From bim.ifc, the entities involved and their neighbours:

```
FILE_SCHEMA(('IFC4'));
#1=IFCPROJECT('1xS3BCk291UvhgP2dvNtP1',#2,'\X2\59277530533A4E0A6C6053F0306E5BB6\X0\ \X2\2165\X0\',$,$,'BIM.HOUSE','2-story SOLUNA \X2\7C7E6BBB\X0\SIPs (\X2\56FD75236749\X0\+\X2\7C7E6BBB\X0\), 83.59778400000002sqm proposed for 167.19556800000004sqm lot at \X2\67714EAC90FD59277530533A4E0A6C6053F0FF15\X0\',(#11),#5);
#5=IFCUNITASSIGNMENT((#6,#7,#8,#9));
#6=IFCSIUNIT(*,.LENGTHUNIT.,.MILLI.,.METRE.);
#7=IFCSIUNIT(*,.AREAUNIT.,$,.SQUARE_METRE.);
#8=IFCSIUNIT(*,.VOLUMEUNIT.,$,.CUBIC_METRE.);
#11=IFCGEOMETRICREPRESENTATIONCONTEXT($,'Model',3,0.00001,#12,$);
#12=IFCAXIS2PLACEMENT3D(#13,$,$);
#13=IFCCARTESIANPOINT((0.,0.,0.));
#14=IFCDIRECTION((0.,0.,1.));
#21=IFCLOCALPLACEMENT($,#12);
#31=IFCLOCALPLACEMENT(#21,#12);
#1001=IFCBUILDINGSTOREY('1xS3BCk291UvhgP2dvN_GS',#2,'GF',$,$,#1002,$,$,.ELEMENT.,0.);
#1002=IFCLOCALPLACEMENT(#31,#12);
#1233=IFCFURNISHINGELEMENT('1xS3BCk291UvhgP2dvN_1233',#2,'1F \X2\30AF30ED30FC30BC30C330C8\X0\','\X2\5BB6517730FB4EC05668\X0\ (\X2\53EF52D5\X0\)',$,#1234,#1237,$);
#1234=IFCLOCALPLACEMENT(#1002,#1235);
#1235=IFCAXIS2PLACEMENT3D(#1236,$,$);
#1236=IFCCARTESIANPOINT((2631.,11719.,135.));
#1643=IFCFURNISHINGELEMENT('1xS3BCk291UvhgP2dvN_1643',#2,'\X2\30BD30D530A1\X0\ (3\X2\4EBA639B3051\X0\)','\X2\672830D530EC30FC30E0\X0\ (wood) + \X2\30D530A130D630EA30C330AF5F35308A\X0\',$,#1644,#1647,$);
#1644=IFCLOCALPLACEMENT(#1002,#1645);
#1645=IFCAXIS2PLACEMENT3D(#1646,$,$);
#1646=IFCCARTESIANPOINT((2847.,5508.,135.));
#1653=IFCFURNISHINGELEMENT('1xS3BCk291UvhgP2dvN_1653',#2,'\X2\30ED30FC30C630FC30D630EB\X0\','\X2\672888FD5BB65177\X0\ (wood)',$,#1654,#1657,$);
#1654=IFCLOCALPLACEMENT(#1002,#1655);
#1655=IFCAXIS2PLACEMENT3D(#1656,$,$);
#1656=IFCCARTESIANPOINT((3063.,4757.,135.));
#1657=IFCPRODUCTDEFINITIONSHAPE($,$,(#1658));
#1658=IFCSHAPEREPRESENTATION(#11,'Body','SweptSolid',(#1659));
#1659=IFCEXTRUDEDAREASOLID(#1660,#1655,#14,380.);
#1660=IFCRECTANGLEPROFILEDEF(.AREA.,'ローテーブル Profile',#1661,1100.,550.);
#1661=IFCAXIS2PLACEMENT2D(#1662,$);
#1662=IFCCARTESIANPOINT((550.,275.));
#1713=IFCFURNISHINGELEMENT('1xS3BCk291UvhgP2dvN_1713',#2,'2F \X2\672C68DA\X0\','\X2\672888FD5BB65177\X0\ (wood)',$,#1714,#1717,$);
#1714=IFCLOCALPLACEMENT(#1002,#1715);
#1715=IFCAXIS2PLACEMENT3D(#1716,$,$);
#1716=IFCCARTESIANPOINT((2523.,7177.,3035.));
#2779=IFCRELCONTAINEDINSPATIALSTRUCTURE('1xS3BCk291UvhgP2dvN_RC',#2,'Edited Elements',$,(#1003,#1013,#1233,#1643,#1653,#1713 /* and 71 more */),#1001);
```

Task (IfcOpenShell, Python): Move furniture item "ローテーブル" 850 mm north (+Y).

```python
import ifcopenshell
import ifcopenshell.api.geometry
import ifcopenshell.util.placement

model = ifcopenshell.open("bim.ifc")

item = model.by_id(1653)
matrix = ifcopenshell.util.placement.get_local_placement(item.ObjectPlacement)
matrix[1, 3] += 850.0
ifcopenshell.api.geometry.edit_object_placement(model, product=item, matrix=matrix, is_si=False)

print(ifcopenshell.util.placement.get_local_placement(item.ObjectPlacement).round(3) + 0.0)

model.write("bim_v2.ifc")
```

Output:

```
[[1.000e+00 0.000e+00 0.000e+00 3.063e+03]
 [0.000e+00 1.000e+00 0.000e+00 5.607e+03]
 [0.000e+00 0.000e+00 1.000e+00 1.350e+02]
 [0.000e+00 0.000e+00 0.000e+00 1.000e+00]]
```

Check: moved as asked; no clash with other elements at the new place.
